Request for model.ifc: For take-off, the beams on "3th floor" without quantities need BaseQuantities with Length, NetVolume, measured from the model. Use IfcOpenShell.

First a look at what the model holds.

```python
import ifcopenshell
import ifcopenshell.util.element
import ifcopenshell.util.unit

model = ifcopenshell.open("model.ifc")
print(model.schema)
for unit_type in ("LENGTHUNIT", "AREAUNIT", "VOLUMEUNIT"):
    print(unit_type, ifcopenshell.util.unit.calculate_unit_scale(model, unit_type))
storey = next(s for s in model.by_type("IfcBuildingStorey") if s.Name == "3th floor")
beams = [e for e in ifcopenshell.util.element.get_decomposition(storey) if e.is_a("IfcBeam")]
for e in sorted(beams, key=lambda e: e.id()):
    print(e.id(), e.is_a(), e.Name, list(ifcopenshell.util.element.get_psets(e, qtos_only=True)), sep=" | ")
```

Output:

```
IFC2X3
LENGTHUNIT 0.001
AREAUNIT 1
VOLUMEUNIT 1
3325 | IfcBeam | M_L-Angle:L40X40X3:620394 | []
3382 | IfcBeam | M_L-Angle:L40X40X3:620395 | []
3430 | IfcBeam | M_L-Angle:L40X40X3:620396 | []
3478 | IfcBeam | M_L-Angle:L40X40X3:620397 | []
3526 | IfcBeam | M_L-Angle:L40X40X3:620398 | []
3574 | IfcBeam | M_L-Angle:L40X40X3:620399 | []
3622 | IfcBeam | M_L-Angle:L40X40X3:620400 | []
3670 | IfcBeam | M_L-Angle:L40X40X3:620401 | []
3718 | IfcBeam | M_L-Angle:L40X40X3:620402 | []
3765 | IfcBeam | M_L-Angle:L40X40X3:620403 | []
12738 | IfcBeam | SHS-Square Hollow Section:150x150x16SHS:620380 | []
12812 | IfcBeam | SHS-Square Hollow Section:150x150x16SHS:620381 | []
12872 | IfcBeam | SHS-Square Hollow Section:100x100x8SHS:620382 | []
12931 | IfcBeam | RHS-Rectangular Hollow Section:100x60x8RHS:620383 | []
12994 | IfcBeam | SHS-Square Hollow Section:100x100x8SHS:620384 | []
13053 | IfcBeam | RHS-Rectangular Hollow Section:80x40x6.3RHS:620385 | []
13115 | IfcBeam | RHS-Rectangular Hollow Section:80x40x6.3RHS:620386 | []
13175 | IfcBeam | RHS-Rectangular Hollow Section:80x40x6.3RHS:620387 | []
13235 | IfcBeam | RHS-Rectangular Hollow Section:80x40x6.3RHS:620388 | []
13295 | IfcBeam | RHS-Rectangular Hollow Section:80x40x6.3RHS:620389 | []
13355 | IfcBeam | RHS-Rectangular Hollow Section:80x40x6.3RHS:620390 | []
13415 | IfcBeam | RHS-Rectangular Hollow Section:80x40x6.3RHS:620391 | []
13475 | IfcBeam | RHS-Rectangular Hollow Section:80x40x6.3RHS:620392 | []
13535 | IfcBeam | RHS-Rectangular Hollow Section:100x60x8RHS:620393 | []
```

```python
import ifcopenshell
import ifcopenshell.api.pset
import ifcopenshell.geom
import ifcopenshell.util.element
import ifcopenshell.util.shape
import ifcopenshell.util.unit

model = ifcopenshell.open("model.ifc")
unit_scale = ifcopenshell.util.unit.calculate_unit_scale(model)
volume_scale = ifcopenshell.util.unit.calculate_unit_scale(model, "VOLUMEUNIT")
settings = ifcopenshell.geom.settings()

storey = next(s for s in model.by_type("IfcBuildingStorey") if s.Name == "3th floor")
beams = [e for e in ifcopenshell.util.element.get_decomposition(storey) if e.is_a("IfcBeam")]

for e in sorted(beams, key=lambda e: e.id()):
    if ifcopenshell.util.element.get_psets(e, qtos_only=True, should_inherit=False):
        continue
    # Geometry comes back in metres, in the element's own axes.
    shape = ifcopenshell.geom.create_shape(settings, e)
    values = {
        "Length": ifcopenshell.util.shape.get_max_xyz(shape.geometry) / unit_scale,
        "NetVolume": ifcopenshell.util.shape.get_volume(shape.geometry) / volume_scale,
    }
    qto = ifcopenshell.api.pset.add_qto(model, product=e, name="BaseQuantities")
    ifcopenshell.api.pset.edit_qto(model, qto=qto, properties=values)
    print(e.id(), {k: round(v, 3) for k, v in values.items()})

model.write("model_v2.ifc")
```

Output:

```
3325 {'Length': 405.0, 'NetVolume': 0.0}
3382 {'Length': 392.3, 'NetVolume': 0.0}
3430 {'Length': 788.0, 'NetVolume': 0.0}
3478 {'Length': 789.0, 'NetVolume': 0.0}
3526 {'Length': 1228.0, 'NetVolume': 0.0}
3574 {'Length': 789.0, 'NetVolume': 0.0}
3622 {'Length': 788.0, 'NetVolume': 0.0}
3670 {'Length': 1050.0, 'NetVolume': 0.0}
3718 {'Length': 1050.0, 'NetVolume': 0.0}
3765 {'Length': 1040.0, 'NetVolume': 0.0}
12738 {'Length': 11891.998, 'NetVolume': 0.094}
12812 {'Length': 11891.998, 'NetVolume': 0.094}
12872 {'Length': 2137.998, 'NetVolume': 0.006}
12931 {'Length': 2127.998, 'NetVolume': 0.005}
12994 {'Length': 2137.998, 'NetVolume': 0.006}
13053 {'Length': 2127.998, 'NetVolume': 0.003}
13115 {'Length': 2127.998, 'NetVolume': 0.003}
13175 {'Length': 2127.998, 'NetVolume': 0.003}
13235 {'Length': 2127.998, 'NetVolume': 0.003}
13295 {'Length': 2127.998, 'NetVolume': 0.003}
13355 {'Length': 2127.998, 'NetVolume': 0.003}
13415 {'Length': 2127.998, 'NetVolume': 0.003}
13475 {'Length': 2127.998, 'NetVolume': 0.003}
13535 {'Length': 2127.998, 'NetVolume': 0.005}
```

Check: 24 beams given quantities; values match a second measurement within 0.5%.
